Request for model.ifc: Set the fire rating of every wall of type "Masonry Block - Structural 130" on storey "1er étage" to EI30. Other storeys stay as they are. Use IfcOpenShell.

First a look at what the model holds.

```python
import ifcopenshell
import ifcopenshell.util.element

model = ifcopenshell.open("model.ifc")
print(model.schema)
storey = next(s for s in model.by_type("IfcBuildingStorey") if s.Name == "1er étage")
walls = [e for e in ifcopenshell.util.element.get_decomposition(storey) if e.is_a("IfcWall")]
seen = {}
for e in walls:
    element_type = ifcopenshell.util.element.get_type(e)
    key = (element_type.Name if element_type != e and element_type else None, ifcopenshell.util.element.get_pset(e, "Pset_WallCommon", "FireRating"))
    seen[key] = seen.get(key, 0) + 1
for (name, value), count in sorted(seen.items(), key=str):
    print(count, "x", name, "|", value)
```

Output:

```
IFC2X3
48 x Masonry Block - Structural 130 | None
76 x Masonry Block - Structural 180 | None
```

```python
import ifcopenshell
import ifcopenshell.api.pset
import ifcopenshell.util.element

model = ifcopenshell.open("model.ifc")

storey = next(s for s in model.by_type("IfcBuildingStorey") if s.Name == "1er étage")
walls = [e for e in ifcopenshell.util.element.get_decomposition(storey) if e.is_a("IfcWall")]

count = 0
for e in walls:
    element_type = ifcopenshell.util.element.get_type(e)
    if element_type in (None, e) or element_type.Name != "Masonry Block - Structural 130":
        continue
    # add_pset returns the element's existing set when there is one.
    pset = ifcopenshell.api.pset.add_pset(model, product=e, name="Pset_WallCommon")
    ifcopenshell.api.pset.edit_pset(model, pset=pset, properties={"FireRating": "EI30"})
    count += 1

print(count, "walls updated")

model.write("model_edited.ifc")
```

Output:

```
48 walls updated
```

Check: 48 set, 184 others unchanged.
